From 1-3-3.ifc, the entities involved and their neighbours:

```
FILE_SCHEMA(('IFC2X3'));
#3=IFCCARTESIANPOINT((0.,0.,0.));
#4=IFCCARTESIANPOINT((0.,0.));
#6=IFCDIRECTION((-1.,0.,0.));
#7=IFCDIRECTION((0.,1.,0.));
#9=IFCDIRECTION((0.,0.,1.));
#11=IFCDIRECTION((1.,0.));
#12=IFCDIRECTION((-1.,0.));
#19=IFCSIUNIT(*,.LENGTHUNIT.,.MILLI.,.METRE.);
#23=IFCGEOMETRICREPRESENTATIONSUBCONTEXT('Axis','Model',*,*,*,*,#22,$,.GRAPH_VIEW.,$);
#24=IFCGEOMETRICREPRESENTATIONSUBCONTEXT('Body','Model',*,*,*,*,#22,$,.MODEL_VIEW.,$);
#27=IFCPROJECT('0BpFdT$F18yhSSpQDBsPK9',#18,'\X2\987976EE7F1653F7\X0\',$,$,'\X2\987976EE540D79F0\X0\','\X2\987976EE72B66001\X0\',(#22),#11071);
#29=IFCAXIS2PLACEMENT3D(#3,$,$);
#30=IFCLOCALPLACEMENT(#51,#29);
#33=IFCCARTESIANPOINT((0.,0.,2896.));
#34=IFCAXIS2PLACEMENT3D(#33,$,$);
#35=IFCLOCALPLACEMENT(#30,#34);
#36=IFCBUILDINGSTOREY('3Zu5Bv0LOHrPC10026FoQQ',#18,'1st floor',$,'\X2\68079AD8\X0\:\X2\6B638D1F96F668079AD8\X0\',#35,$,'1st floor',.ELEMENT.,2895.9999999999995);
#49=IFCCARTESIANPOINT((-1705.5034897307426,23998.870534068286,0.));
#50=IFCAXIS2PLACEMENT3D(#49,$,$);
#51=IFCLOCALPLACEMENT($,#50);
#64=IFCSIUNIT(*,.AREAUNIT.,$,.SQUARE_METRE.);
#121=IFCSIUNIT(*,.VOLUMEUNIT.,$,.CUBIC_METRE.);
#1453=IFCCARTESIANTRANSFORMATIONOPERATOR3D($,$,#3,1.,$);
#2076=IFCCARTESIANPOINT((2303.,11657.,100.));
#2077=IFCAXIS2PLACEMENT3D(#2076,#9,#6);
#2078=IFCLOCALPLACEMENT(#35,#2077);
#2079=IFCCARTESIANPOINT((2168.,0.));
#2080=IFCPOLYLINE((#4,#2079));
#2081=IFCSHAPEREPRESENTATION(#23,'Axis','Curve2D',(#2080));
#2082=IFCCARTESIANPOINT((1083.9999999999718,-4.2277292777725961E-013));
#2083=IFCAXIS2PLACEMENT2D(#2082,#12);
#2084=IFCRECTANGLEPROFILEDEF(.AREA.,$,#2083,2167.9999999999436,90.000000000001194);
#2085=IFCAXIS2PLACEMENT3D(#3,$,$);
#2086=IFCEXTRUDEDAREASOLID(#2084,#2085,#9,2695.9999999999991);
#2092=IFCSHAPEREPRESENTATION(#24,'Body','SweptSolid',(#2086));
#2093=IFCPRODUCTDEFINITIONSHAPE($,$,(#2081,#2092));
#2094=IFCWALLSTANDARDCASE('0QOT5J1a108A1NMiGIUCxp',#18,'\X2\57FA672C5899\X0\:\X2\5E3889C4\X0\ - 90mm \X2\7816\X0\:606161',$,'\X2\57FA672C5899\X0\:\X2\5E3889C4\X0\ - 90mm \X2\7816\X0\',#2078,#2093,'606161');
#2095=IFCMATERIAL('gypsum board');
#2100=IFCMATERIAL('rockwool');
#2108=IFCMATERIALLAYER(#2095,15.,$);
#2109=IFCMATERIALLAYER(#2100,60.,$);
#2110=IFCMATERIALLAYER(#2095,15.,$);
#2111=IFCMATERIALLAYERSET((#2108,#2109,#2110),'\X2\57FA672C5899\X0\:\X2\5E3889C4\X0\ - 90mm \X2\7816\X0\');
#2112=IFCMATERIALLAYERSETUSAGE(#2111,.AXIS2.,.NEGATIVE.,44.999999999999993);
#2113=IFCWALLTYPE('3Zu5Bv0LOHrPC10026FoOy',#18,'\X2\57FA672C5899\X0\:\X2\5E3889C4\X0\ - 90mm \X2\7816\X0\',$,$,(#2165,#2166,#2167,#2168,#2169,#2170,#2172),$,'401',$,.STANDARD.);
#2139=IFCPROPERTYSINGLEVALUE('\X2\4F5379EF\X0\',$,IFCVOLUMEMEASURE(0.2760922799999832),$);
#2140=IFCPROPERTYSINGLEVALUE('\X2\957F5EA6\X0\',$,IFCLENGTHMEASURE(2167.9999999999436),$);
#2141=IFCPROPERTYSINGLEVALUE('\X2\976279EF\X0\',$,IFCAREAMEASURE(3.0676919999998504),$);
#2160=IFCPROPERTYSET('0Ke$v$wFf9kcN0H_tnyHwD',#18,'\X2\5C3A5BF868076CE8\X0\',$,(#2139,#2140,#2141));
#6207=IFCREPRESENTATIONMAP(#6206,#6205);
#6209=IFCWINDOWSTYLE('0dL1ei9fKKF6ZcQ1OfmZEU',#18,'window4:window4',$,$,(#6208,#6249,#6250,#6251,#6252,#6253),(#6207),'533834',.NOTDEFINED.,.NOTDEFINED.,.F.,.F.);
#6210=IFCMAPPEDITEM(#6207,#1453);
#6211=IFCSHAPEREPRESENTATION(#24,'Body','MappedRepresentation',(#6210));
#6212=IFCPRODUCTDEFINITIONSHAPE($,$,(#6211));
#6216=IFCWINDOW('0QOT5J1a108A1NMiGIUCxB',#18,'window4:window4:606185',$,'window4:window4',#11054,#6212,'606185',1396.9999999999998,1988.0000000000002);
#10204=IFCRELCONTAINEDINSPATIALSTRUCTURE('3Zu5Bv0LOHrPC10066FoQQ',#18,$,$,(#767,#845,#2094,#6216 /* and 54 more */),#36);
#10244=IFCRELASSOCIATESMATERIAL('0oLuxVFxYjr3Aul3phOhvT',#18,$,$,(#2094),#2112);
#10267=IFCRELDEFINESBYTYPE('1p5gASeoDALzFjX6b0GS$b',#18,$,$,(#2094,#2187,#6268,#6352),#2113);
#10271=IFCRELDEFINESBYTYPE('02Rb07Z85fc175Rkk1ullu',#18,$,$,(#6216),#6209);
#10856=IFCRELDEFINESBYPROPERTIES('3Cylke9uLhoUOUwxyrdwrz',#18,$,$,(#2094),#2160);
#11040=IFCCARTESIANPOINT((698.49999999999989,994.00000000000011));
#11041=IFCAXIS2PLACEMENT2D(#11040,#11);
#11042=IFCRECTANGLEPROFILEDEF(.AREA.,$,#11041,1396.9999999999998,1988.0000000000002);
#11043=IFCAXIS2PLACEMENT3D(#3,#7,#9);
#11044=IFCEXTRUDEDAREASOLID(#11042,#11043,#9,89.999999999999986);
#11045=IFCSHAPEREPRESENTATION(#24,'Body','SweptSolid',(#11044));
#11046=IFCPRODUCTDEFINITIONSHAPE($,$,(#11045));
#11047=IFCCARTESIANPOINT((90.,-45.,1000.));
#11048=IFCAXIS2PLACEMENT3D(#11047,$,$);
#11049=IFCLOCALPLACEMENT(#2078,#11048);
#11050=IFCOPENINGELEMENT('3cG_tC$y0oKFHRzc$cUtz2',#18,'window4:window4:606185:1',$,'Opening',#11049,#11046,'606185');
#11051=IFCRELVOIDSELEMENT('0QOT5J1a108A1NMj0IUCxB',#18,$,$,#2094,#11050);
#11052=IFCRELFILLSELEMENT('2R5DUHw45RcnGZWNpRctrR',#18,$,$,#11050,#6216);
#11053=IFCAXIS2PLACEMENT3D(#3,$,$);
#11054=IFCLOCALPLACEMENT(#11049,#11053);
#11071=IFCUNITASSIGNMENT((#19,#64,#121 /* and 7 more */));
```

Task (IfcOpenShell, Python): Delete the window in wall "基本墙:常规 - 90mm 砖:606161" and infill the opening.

```python
import ifcopenshell
import ifcopenshell.api.feature
import ifcopenshell.api.pset
import ifcopenshell.api.root
import ifcopenshell.geom
import ifcopenshell.util.element
import ifcopenshell.util.shape
import ifcopenshell.util.unit

model = ifcopenshell.open("1-3-3.ifc")
area_scale = ifcopenshell.util.unit.calculate_unit_scale(model, "AREAUNIT")
volume_scale = ifcopenshell.util.unit.calculate_unit_scale(model, "VOLUMEUNIT")
settings = ifcopenshell.geom.settings()


def volume(element):
    """Net volume in cubic metres, openings subtracted."""
    shape = ifcopenshell.geom.create_shape(settings, element)
    return ifcopenshell.util.shape.get_volume(shape.geometry)


window = model.by_guid("0QOT5J1a108A1NMiGIUCxB")
opening = window.FillsVoids[0].RelatingOpeningElement
wall = opening.VoidsElements[0].RelatingBuildingElement
before = volume(wall)

ifcopenshell.api.root.remove_product(model, product=window)
ifcopenshell.api.feature.remove_feature(model, feature=opening)

after = volume(wall)
thickness = 0.09  # wall thickness in metres

# Update the wall's stored quantities.
pset = model.by_id(ifcopenshell.util.element.get_pset(wall, "尺寸标注", should_inherit=False)["id"])
ifcopenshell.api.pset.edit_pset(model, pset=pset, properties={
    "体积": model.create_entity("IfcVolumeMeasure", after / volume_scale),
    "面积": model.create_entity("IfcAreaMeasure", after / thickness / area_scale),
})

print(f"wall volume {before:.3f} -> {after:.3f} m3")

model.write("1-3-3_edited.ifc")
```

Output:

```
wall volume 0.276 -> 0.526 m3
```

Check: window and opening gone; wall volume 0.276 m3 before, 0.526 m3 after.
